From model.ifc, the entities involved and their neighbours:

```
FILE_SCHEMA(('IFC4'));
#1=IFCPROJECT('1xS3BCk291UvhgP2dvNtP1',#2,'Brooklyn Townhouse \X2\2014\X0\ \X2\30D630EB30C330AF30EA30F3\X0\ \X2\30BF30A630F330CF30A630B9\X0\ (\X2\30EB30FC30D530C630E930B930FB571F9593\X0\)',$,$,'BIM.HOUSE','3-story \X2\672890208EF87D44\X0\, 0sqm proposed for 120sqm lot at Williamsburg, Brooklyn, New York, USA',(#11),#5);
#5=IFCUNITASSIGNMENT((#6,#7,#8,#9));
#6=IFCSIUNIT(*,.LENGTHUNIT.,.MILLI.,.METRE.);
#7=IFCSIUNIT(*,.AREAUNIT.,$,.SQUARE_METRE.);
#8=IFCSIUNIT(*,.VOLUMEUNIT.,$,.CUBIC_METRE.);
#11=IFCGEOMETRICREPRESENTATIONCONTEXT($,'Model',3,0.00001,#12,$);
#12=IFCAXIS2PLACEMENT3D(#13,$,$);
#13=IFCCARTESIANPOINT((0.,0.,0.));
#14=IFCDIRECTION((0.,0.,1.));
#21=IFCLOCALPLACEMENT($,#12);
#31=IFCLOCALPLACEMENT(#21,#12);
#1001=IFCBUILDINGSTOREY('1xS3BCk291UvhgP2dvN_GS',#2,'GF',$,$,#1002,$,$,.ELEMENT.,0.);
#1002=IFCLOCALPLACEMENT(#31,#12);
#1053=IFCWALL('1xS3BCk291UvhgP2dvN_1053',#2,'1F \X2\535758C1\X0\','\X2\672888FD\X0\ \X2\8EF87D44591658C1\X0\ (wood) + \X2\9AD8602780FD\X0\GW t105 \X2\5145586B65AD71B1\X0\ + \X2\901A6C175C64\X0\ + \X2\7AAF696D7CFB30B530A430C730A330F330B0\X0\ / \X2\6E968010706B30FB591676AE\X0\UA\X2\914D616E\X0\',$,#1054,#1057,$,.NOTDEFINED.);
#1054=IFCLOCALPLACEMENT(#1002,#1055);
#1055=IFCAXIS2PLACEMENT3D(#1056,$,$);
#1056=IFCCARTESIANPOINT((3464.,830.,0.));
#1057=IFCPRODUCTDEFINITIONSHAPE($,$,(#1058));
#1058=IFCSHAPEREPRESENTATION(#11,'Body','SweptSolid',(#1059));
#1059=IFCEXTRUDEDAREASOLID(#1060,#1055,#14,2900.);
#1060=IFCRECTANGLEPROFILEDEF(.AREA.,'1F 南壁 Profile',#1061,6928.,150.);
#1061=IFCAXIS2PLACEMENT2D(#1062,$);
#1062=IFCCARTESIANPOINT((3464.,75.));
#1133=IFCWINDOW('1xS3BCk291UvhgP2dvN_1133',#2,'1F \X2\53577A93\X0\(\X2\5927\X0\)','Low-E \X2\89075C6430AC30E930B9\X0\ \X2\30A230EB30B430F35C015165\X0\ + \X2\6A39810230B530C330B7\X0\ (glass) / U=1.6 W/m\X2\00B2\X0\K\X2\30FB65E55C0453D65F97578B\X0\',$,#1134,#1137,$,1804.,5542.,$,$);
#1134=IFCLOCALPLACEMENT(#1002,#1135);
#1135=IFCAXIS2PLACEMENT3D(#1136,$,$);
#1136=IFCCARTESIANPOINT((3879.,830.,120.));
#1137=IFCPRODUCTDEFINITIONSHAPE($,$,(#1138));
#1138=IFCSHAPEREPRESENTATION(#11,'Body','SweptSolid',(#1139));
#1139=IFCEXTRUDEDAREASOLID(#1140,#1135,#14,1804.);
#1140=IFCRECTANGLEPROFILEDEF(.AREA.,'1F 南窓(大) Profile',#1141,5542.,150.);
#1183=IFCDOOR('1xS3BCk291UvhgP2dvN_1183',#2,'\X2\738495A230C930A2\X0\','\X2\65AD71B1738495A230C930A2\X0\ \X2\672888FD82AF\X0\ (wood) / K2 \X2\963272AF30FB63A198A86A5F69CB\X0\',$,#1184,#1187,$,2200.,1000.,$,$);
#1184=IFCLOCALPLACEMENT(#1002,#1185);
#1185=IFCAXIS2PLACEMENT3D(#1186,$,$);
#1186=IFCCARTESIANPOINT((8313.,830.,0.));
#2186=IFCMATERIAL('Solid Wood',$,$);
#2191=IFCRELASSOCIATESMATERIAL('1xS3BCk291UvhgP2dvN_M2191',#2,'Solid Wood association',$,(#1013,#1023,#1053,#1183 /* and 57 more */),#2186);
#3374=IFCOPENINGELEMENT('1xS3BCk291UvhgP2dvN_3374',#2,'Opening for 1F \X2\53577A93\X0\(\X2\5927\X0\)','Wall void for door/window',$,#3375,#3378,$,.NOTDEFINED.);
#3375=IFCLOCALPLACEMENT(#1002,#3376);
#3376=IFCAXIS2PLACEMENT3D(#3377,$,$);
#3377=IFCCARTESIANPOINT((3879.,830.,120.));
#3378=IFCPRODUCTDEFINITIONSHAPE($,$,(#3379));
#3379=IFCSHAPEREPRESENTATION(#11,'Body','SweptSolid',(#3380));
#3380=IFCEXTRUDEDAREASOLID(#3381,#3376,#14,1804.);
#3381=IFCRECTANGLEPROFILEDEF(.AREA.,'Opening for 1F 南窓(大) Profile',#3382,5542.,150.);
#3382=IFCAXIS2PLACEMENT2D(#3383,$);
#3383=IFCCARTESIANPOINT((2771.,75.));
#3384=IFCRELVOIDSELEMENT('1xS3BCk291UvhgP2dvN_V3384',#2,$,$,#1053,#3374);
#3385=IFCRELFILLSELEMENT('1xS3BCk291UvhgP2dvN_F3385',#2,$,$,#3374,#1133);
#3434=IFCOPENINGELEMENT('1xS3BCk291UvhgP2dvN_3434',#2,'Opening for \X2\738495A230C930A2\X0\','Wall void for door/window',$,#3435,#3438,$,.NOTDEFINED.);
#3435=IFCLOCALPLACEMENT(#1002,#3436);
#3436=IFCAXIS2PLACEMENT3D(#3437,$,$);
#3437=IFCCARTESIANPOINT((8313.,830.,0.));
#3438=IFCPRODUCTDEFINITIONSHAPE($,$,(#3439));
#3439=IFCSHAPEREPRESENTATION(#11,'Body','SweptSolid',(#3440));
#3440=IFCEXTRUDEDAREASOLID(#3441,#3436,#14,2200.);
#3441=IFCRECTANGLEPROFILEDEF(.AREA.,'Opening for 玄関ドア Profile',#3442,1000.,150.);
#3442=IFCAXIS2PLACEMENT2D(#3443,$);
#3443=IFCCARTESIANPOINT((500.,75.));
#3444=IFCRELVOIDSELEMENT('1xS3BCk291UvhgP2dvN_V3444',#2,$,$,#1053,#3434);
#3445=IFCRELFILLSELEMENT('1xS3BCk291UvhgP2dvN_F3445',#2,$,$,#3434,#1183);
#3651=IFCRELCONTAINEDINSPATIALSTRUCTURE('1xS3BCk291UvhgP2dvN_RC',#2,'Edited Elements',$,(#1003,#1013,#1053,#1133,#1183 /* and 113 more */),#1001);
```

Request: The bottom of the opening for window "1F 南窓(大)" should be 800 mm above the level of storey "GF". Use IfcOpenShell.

```python
import numpy as np
import ifcopenshell
import ifcopenshell.api.geometry
import ifcopenshell.geom
import ifcopenshell.util.element
import ifcopenshell.util.placement
import ifcopenshell.util.shape
import ifcopenshell.util.unit

model = ifcopenshell.open("model.ifc")
unit_scale = ifcopenshell.util.unit.calculate_unit_scale(model)

window = model.by_guid("1xS3BCk291UvhgP2dvN_1133")
opening = window.FillsVoids[0].RelatingOpeningElement
storey = ifcopenshell.util.element.get_container(window, ifc_class="IfcBuildingStorey")
level = ifcopenshell.util.placement.get_local_placement(storey.ObjectPlacement)[2, 3]

# The opening's origin need not be at the sill, so measure its lowest point.
shape = ifcopenshell.geom.create_shape(ifcopenshell.geom.settings(), opening)
bottom = ifcopenshell.util.shape.get_shape_bottom_elevation(shape, shape.geometry) / unit_scale
dz = level + 0.8 / unit_scale - bottom

shift = np.array([0.0, 0.0, dz])
# The window is not placed relative to its opening, so move both.
for product in (opening, window):
    matrix = ifcopenshell.util.placement.get_local_placement(product.ObjectPlacement)
    matrix[:3, 3] += shift
    ifcopenshell.api.geometry.edit_object_placement(model, product=product, matrix=matrix, is_si=False)

print(f"moved by {dz * unit_scale:+.3f} m")

model.write("model_edited.ifc")
```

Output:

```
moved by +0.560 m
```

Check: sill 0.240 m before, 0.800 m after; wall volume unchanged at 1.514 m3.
